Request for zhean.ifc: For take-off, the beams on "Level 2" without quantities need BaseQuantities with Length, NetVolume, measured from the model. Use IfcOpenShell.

First a look at what the model holds.

```python
import ifcopenshell
import ifcopenshell.util.element
import ifcopenshell.util.unit

model = ifcopenshell.open("zhean.ifc")
print(model.schema)
for unit_type in ("LENGTHUNIT", "AREAUNIT", "VOLUMEUNIT"):
    print(unit_type, ifcopenshell.util.unit.calculate_unit_scale(model, unit_type))
storey = next(s for s in model.by_type("IfcBuildingStorey") if s.Name == "Level 2")
beams = [e for e in ifcopenshell.util.element.get_decomposition(storey) if e.is_a("IfcBeam")]
for e in sorted(beams, key=lambda e: e.id()):
    print(e.id(), e.is_a(), e.Name, list(ifcopenshell.util.element.get_psets(e, qtos_only=True)), sep=" | ")
```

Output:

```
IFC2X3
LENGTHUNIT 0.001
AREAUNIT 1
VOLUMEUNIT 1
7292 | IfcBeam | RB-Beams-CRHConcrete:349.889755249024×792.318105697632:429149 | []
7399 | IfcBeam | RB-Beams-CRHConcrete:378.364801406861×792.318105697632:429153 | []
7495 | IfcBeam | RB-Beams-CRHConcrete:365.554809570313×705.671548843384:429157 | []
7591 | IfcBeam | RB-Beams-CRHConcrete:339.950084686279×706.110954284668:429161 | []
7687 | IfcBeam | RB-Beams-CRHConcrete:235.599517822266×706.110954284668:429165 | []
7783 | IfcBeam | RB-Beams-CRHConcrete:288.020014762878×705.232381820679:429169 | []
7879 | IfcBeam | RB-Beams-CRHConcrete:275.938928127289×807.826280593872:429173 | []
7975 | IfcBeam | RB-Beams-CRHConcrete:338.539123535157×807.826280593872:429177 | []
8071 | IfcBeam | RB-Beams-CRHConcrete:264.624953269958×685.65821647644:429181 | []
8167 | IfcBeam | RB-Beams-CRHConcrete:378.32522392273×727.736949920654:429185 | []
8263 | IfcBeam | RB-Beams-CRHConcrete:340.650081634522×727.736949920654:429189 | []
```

```python
import ifcopenshell
import ifcopenshell.api.pset
import ifcopenshell.geom
import ifcopenshell.util.element
import ifcopenshell.util.shape
import ifcopenshell.util.unit

model = ifcopenshell.open("zhean.ifc")
unit_scale = ifcopenshell.util.unit.calculate_unit_scale(model)
volume_scale = ifcopenshell.util.unit.calculate_unit_scale(model, "VOLUMEUNIT")
settings = ifcopenshell.geom.settings()

storey = next(s for s in model.by_type("IfcBuildingStorey") if s.Name == "Level 2")
beams = [e for e in ifcopenshell.util.element.get_decomposition(storey) if e.is_a("IfcBeam")]

for e in sorted(beams, key=lambda e: e.id()):
    if ifcopenshell.util.element.get_psets(e, qtos_only=True, should_inherit=False):
        continue
    # Geometry comes back in metres, in the element's own axes.
    shape = ifcopenshell.geom.create_shape(settings, e)
    values = {
        "Length": ifcopenshell.util.shape.get_max_xyz(shape.geometry) / unit_scale,
        "NetVolume": ifcopenshell.util.shape.get_volume(shape.geometry) / volume_scale,
    }
    qto = ifcopenshell.api.pset.add_qto(model, product=e, name="BaseQuantities")
    ifcopenshell.api.pset.edit_qto(model, qto=qto, properties=values)
    print(e.id(), {k: round(v, 3) for k, v in values.items()})

model.write("zhean_v2.ifc")
```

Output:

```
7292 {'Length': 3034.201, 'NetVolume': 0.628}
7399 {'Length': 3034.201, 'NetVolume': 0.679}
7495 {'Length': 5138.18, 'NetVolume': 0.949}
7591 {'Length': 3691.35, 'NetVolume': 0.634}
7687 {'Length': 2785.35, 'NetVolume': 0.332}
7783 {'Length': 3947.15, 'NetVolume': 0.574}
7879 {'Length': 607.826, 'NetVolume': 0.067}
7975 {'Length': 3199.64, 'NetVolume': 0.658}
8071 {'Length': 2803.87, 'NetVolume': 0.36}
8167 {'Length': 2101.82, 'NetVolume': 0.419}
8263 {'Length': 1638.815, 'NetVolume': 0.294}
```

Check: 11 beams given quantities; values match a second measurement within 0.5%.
